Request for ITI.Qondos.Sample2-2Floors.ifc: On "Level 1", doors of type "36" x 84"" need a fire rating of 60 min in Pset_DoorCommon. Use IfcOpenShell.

First a look at what the model holds.

```python
import ifcopenshell
import ifcopenshell.util.element

model = ifcopenshell.open("ITI.Qondos.Sample2-2Floors.ifc")
print(model.schema)
storey = next(s for s in model.by_type("IfcBuildingStorey") if s.Name == "Level 1")
doors = [e for e in ifcopenshell.util.element.get_decomposition(storey) if e.is_a("IfcDoor")]
seen = {}
for e in doors:
    element_type = ifcopenshell.util.element.get_type(e)
    key = (element_type.Name if element_type != e and element_type else None, ifcopenshell.util.element.get_pset(e, "Pset_DoorCommon", "FireRating"))
    seen[key] = seen.get(key, 0) + 1
for (name, value), count in sorted(seen.items(), key=str):
    print(count, "x", name, "|", value)
```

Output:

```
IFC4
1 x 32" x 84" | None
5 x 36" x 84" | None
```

```python
import ifcopenshell
import ifcopenshell.api.pset
import ifcopenshell.util.element

model = ifcopenshell.open("ITI.Qondos.Sample2-2Floors.ifc")

storey = next(s for s in model.by_type("IfcBuildingStorey") if s.Name == "Level 1")
doors = [e for e in ifcopenshell.util.element.get_decomposition(storey) if e.is_a("IfcDoor")]

count = 0
for e in doors:
    element_type = ifcopenshell.util.element.get_type(e)
    if element_type in (None, e) or element_type.Name != '36" x 84"':
        continue
    # add_pset returns the element's existing set when there is one.
    pset = ifcopenshell.api.pset.add_pset(model, product=e, name="Pset_DoorCommon")
    ifcopenshell.api.pset.edit_pset(model, pset=pset, properties={"FireRating": "60 min"})
    count += 1

print(count, "doors updated")

model.write("ITI.Qondos.Sample2-2Floors_v2.ifc")
```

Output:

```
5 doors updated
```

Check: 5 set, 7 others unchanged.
